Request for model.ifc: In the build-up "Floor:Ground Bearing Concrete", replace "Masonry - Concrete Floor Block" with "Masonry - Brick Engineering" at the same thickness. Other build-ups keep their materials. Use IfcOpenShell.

First a look at what the model holds.

```python
import ifcopenshell
import ifcopenshell.util.element

model = ifcopenshell.open("model.ifc")
print(model.schema)
for layer_set in model.by_type("IfcMaterialLayerSet"):
    if layer_set.LayerSetName == "Floor:Ground Bearing Concrete":
        for layer in layer_set.MaterialLayers:
            print(layer.id(), layer.Material and layer.Material.Name, layer.LayerThickness, sep=" | ")
        print(len(ifcopenshell.util.element.get_elements_by_material(model, layer_set)), "elements and types use it")
print(sorted(m.Name for m in model.by_type("IfcMaterial") if m.Name)[:60])
```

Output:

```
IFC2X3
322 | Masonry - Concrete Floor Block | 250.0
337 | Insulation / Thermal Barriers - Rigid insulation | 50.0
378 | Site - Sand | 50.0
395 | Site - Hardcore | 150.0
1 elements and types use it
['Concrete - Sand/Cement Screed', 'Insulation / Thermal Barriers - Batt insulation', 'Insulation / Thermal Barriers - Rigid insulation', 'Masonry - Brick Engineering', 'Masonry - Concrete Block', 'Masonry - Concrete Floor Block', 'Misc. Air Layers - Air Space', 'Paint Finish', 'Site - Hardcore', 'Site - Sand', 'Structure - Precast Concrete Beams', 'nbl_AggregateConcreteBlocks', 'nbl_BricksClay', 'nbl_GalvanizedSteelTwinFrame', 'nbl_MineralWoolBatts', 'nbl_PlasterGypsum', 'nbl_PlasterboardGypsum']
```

```python
import ifcopenshell
import ifcopenshell.api.material

model = ifcopenshell.open("model.ifc")

layer_set = next(s for s in model.by_type("IfcMaterialLayerSet") if s.LayerSetName == "Floor:Ground Bearing Concrete")
layer = next(l for l in layer_set.MaterialLayers if l.Material and l.Material.Name == "Masonry - Concrete Floor Block")
material = next(m for m in model.by_type("IfcMaterial") if m.Name == "Masonry - Brick Engineering")

# Point this one layer at the other material; renaming the old one would change it everywhere.
ifcopenshell.api.material.edit_layer(model, layer=layer, attributes={}, material=material)

print([l.Material.Name if l.Material else None for l in layer_set.MaterialLayers])

model.write("model_rev.ifc")
```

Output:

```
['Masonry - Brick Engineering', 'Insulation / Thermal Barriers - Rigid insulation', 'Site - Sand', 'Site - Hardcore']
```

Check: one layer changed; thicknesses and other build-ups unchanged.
